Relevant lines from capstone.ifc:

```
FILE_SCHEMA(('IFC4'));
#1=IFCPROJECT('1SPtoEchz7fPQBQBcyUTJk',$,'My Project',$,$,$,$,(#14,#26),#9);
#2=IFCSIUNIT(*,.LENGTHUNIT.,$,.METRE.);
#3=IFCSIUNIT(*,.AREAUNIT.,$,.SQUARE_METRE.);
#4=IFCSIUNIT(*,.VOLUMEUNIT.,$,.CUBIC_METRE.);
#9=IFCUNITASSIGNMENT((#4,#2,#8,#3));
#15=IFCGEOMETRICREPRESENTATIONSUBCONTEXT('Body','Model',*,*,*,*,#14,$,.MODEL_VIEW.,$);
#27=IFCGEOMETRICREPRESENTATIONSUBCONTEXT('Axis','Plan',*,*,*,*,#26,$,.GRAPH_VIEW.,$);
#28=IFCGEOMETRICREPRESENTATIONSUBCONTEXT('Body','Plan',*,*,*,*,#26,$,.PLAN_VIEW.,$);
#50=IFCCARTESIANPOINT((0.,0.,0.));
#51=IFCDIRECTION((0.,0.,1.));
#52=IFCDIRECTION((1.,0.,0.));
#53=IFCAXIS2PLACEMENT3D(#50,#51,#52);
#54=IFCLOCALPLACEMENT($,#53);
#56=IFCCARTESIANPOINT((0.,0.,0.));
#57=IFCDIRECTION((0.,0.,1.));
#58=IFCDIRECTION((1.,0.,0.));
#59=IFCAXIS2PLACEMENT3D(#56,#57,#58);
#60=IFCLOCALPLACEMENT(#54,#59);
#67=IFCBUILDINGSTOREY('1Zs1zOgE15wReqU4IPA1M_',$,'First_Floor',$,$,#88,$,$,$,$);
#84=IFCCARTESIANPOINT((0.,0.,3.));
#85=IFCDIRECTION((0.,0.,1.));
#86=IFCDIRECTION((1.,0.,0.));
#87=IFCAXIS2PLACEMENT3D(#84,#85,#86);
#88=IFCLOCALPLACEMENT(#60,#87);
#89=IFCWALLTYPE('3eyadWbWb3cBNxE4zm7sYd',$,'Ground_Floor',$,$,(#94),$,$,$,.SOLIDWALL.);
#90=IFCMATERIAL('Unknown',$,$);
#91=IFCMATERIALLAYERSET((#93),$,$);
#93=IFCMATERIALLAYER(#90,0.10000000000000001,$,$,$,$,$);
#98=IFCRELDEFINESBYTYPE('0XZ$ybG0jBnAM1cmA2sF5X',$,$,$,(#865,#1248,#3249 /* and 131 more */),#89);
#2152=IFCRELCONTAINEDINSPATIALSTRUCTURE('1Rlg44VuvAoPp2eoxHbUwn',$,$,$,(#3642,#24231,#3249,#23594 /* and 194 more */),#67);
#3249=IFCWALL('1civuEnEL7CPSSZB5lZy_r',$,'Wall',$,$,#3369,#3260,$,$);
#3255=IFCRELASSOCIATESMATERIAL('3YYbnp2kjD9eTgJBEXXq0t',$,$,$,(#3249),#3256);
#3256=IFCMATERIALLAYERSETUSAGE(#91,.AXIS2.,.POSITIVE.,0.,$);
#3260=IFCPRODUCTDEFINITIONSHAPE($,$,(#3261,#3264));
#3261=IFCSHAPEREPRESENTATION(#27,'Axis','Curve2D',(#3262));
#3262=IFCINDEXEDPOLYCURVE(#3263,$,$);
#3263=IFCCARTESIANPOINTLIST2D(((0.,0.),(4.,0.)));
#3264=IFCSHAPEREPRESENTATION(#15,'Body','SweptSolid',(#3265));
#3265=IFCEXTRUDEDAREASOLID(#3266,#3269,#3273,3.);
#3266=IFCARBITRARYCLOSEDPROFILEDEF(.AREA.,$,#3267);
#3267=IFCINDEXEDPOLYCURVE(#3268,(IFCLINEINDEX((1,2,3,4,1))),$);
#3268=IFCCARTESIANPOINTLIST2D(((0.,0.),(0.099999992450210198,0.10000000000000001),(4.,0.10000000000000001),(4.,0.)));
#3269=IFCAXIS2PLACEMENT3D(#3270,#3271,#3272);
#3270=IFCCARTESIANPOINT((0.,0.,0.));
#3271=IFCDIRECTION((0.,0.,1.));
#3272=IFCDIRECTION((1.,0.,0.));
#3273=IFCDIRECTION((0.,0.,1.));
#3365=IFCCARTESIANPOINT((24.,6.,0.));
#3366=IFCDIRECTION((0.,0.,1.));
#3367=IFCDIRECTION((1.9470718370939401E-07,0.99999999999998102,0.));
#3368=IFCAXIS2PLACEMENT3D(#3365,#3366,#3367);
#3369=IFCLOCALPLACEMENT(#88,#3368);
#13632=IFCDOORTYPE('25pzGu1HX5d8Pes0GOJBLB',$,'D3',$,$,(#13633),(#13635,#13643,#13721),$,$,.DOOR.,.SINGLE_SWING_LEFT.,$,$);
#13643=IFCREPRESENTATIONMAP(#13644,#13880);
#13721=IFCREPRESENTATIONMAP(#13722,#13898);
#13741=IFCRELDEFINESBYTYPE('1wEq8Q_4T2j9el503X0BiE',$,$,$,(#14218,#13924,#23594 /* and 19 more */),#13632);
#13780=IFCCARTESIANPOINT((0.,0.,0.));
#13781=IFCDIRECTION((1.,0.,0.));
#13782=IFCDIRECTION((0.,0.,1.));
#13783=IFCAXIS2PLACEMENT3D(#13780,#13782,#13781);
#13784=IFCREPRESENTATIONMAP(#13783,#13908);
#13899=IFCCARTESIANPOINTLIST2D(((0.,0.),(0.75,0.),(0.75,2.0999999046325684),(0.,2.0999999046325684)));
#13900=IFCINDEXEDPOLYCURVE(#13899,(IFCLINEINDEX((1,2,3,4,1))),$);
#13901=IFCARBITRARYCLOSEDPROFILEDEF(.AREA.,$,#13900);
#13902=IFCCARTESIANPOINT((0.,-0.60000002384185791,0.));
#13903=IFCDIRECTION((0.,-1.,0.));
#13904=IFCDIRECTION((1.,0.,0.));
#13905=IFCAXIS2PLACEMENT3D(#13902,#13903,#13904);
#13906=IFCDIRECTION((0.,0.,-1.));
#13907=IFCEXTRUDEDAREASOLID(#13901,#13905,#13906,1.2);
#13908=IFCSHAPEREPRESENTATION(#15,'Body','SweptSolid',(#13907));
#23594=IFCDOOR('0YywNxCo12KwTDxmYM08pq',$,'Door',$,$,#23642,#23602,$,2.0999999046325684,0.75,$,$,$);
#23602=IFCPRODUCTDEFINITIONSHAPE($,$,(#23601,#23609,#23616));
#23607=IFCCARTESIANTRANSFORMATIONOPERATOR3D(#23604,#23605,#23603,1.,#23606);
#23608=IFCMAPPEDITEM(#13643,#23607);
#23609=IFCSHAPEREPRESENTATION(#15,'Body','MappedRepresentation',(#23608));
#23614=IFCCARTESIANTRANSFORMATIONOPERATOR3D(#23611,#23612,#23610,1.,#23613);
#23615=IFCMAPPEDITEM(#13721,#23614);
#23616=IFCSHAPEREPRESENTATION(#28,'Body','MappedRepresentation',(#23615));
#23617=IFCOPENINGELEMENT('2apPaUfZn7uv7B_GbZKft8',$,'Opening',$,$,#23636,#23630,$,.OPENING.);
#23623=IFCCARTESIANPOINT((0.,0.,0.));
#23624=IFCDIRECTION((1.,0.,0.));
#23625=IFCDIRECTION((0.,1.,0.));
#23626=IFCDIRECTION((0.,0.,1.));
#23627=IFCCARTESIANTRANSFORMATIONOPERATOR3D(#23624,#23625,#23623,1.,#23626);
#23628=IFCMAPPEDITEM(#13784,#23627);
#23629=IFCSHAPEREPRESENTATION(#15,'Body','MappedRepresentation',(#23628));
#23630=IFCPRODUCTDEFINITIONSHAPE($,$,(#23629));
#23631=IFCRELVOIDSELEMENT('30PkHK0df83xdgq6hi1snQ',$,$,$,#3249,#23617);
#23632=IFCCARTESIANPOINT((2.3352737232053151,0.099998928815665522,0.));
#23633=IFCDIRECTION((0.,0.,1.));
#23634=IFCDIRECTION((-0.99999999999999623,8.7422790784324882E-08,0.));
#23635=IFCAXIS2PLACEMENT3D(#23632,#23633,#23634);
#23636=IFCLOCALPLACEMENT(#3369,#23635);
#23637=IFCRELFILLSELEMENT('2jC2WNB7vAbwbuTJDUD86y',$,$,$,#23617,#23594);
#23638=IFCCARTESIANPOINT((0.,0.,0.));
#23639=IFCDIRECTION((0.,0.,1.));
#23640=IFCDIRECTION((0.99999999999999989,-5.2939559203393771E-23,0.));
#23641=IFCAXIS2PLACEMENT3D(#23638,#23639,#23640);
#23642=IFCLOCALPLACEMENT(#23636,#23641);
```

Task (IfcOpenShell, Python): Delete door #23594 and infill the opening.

```python
import ifcopenshell
import ifcopenshell.api.feature
import ifcopenshell.api.root
import ifcopenshell.geom
import ifcopenshell.util.shape

model = ifcopenshell.open("capstone.ifc")
settings = ifcopenshell.geom.settings()


def volume(element):
    """Net volume in cubic metres, openings subtracted."""
    shape = ifcopenshell.geom.create_shape(settings, element)
    return ifcopenshell.util.shape.get_volume(shape.geometry)


door = model.by_id(23594)
opening = door.FillsVoids[0].RelatingOpeningElement
wall = opening.VoidsElements[0].RelatingBuildingElement
before = volume(wall)

ifcopenshell.api.root.remove_product(model, product=door)
ifcopenshell.api.feature.remove_feature(model, feature=opening)

after = volume(wall)

print(f"wall volume {before:.3f} -> {after:.3f} m3")

model.write("capstone-out.ifc")
```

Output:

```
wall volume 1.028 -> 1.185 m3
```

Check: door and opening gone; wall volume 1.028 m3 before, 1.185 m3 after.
